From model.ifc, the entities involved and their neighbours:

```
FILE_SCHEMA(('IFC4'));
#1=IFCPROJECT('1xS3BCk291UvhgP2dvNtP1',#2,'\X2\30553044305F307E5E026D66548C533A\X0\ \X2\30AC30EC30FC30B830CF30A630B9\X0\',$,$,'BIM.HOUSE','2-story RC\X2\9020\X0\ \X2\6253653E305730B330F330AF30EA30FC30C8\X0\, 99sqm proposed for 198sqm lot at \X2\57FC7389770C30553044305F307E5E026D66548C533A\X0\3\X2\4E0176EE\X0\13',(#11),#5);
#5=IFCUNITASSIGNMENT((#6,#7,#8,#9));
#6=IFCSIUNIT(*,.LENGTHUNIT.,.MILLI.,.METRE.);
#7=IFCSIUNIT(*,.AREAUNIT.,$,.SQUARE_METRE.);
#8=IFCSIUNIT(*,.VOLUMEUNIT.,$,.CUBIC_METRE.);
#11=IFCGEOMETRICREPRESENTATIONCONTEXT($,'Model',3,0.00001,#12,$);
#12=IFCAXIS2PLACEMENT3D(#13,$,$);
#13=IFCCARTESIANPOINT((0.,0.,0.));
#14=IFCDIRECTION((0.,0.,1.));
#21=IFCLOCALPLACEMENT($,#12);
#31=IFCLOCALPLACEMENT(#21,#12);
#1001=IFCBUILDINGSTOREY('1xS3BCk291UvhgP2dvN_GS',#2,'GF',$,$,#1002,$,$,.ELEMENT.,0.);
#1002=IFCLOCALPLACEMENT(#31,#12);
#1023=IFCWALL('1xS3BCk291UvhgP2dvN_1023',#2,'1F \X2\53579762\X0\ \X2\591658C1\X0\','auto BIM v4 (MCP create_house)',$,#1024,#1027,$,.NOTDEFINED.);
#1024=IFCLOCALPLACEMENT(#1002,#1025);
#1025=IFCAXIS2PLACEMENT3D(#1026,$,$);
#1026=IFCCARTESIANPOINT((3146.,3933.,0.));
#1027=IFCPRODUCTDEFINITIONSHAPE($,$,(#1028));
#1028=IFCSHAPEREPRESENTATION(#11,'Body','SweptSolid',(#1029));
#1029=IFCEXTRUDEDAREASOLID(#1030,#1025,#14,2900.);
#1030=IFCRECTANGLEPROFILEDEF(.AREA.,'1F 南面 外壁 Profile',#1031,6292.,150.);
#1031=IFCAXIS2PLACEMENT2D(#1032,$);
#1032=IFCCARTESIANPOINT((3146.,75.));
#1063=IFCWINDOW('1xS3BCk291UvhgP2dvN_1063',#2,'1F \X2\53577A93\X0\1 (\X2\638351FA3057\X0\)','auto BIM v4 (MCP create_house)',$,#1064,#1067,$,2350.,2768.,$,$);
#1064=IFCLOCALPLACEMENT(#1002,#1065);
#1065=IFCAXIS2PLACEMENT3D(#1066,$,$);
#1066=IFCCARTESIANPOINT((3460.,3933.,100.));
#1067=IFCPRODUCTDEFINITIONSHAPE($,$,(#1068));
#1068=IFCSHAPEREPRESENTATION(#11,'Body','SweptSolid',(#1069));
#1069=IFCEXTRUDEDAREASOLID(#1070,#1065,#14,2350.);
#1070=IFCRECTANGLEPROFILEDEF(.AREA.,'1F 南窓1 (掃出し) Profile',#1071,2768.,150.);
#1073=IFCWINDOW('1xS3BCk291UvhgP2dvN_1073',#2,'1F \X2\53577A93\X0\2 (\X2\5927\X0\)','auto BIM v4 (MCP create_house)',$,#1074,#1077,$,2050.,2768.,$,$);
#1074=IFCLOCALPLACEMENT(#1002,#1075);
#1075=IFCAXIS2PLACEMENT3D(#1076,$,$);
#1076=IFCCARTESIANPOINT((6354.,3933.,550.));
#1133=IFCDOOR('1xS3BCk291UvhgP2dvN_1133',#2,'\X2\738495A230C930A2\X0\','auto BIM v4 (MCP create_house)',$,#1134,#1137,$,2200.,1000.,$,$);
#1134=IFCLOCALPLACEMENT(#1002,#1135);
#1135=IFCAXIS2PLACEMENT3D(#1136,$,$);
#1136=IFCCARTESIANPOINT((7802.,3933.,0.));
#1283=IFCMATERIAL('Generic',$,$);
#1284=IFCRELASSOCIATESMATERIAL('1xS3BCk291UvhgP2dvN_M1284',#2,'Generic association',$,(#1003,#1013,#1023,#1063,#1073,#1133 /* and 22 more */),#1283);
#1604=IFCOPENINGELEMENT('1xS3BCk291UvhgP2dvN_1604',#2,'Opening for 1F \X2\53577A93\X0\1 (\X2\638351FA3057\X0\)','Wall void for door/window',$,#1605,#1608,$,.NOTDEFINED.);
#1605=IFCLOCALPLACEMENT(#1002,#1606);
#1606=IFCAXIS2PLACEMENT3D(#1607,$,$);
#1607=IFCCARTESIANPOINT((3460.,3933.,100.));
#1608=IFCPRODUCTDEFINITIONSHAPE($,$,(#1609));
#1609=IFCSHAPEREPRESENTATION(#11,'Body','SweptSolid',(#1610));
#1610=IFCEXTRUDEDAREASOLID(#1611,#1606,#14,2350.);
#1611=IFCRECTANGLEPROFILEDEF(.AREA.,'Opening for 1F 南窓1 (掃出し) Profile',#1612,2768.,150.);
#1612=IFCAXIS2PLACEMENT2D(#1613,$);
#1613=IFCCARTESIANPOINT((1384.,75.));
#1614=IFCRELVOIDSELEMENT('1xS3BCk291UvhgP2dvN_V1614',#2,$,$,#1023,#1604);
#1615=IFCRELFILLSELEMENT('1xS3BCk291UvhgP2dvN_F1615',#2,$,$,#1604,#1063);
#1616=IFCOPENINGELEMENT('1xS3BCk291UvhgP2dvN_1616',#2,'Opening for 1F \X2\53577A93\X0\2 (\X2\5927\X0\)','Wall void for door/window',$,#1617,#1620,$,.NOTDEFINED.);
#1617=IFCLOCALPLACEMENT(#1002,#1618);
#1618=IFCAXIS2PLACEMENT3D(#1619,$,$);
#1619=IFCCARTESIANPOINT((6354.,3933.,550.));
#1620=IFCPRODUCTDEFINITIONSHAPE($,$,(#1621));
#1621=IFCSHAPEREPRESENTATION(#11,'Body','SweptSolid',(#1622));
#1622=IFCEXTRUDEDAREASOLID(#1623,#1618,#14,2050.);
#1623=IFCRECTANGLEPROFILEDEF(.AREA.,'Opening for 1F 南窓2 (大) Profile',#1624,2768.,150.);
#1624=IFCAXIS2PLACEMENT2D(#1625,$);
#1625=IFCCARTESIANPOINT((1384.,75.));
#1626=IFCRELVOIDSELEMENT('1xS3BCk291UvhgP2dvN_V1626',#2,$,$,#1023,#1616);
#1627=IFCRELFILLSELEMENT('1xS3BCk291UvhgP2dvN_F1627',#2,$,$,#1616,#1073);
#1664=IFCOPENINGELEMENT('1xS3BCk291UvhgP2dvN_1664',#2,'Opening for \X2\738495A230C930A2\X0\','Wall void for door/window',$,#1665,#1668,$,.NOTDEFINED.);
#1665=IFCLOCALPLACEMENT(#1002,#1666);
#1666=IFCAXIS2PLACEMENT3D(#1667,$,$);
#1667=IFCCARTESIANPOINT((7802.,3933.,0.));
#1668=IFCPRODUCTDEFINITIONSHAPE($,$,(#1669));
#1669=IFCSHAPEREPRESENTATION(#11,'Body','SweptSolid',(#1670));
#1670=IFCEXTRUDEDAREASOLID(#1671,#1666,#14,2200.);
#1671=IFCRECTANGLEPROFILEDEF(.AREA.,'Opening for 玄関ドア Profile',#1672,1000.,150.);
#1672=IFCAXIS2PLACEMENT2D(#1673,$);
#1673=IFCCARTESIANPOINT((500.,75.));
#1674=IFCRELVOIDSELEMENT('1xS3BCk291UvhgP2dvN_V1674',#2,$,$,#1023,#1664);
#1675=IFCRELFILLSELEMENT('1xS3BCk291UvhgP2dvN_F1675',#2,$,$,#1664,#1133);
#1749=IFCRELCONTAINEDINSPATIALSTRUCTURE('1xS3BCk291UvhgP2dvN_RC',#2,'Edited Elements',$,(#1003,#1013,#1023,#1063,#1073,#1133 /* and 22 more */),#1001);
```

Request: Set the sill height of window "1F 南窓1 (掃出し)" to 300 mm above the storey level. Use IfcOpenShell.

```python
import numpy as np
import ifcopenshell
import ifcopenshell.api.geometry
import ifcopenshell.geom
import ifcopenshell.util.element
import ifcopenshell.util.placement
import ifcopenshell.util.shape
import ifcopenshell.util.unit

model = ifcopenshell.open("model.ifc")
unit_scale = ifcopenshell.util.unit.calculate_unit_scale(model)

window = model.by_guid("1xS3BCk291UvhgP2dvN_1063")
opening = window.FillsVoids[0].RelatingOpeningElement
storey = ifcopenshell.util.element.get_container(window, ifc_class="IfcBuildingStorey")
level = ifcopenshell.util.placement.get_local_placement(storey.ObjectPlacement)[2, 3]

# The opening's origin need not be at the sill, so measure its lowest point.
shape = ifcopenshell.geom.create_shape(ifcopenshell.geom.settings(), opening)
bottom = ifcopenshell.util.shape.get_shape_bottom_elevation(shape, shape.geometry) / unit_scale
dz = level + 0.3 / unit_scale - bottom

shift = np.array([0.0, 0.0, dz])
# The window is not placed relative to its opening, so move both.
for product in (opening, window):
    matrix = ifcopenshell.util.placement.get_local_placement(product.ObjectPlacement)
    matrix[:3, 3] += shift
    ifcopenshell.api.geometry.edit_object_placement(model, product=product, matrix=matrix, is_si=False)

print(f"moved by {dz * unit_scale:+.3f} m")

model.write("model_edited.ifc")
```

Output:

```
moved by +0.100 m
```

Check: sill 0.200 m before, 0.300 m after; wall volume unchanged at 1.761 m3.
